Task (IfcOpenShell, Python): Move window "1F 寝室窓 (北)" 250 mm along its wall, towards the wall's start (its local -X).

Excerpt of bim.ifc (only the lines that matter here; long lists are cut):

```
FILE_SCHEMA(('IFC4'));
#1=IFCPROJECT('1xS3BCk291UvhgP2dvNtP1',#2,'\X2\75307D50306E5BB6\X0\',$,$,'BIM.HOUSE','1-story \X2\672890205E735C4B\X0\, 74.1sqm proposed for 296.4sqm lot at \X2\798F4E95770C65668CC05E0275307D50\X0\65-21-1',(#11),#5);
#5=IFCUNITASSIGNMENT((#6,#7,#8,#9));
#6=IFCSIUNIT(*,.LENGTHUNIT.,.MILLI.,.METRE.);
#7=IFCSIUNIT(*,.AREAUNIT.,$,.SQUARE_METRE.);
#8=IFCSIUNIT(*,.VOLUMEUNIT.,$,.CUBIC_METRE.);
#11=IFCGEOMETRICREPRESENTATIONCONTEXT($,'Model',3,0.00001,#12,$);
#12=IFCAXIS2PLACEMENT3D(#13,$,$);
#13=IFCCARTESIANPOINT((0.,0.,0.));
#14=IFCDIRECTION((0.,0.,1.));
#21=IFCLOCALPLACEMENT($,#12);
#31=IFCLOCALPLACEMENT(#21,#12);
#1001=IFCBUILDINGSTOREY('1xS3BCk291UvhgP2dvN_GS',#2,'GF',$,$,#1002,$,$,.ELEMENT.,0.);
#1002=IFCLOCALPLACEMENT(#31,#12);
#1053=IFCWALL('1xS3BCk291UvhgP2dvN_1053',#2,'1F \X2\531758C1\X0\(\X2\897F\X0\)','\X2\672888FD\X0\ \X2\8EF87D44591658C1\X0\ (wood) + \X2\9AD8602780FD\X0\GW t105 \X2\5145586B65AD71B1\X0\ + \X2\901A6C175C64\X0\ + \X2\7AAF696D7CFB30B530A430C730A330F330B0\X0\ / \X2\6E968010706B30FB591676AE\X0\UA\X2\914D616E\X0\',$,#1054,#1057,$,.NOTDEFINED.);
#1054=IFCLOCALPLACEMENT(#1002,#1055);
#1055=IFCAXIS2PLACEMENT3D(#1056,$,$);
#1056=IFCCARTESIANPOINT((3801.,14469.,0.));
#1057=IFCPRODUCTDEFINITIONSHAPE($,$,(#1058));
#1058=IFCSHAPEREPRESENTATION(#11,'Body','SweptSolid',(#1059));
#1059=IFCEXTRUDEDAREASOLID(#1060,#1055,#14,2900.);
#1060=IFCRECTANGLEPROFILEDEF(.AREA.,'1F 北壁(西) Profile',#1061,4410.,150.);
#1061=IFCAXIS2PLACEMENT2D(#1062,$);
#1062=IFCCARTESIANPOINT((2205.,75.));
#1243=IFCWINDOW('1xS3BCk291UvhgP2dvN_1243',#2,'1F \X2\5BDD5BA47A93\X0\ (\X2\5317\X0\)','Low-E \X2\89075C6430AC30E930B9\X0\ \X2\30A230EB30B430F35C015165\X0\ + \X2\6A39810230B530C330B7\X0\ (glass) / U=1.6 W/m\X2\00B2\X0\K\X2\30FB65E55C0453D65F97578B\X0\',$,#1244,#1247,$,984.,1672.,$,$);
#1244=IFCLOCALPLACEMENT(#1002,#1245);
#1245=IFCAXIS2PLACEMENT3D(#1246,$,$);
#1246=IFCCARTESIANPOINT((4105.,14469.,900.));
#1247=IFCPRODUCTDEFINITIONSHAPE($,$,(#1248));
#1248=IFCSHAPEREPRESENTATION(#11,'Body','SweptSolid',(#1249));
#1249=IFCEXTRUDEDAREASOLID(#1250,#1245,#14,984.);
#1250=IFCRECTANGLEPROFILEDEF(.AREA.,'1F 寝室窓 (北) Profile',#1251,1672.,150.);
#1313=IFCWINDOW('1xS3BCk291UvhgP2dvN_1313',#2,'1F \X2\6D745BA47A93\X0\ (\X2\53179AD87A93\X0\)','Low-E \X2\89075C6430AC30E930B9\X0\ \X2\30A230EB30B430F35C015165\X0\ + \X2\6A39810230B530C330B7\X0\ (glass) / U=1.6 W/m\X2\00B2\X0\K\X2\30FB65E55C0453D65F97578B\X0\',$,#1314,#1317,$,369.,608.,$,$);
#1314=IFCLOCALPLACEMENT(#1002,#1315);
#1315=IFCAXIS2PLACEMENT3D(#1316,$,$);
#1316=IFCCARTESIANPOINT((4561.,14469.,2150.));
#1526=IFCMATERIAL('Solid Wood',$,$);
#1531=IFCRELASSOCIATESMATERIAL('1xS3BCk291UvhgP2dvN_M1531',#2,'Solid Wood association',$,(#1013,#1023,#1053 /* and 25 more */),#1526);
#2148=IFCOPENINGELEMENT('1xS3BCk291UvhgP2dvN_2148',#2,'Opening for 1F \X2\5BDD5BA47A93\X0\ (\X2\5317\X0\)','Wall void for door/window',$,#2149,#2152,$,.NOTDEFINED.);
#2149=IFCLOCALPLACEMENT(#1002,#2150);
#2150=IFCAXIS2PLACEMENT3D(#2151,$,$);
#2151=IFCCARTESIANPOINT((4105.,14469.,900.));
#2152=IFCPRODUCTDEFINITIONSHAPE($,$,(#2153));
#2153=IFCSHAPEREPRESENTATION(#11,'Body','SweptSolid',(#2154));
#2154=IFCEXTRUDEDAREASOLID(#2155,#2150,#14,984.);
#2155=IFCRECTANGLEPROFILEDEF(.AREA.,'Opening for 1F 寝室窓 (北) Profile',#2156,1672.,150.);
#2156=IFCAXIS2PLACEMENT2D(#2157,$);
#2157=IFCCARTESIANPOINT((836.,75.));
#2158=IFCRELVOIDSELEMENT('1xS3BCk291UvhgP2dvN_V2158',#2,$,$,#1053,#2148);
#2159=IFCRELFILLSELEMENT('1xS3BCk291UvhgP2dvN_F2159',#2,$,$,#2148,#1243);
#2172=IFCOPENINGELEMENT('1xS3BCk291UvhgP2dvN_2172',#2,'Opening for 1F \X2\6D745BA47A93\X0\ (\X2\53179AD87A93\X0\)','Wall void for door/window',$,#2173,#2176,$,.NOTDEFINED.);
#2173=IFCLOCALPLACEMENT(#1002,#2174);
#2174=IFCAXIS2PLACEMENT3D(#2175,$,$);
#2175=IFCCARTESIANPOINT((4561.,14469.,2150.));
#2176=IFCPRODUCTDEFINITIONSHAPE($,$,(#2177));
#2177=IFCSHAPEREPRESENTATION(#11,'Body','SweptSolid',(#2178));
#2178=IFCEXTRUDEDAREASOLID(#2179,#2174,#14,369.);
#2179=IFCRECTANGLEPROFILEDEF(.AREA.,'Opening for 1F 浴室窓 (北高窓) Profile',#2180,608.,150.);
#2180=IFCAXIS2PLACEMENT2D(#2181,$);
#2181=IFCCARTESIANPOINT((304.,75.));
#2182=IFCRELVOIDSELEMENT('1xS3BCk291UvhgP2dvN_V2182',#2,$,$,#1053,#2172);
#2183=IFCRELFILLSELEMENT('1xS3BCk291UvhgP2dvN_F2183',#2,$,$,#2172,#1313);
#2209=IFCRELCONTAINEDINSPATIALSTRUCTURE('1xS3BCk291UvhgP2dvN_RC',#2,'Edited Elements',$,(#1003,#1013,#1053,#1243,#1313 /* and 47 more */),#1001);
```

```python
import ifcopenshell
import ifcopenshell.api.geometry
import ifcopenshell.util.placement
import ifcopenshell.util.unit

model = ifcopenshell.open("bim.ifc")
unit_scale = ifcopenshell.util.unit.calculate_unit_scale(model)

window = model.by_id(1243)
opening = window.FillsVoids[0].RelatingOpeningElement
wall = opening.VoidsElements[0].RelatingBuildingElement

wall_matrix = ifcopenshell.util.placement.get_local_placement(wall.ObjectPlacement)
shift = wall_matrix[:3, 0] * -0.25 / unit_scale
before = ifcopenshell.util.placement.get_local_placement(window.ObjectPlacement)[:3, 3].copy()

# The window is not placed relative to its opening, so move both.
for product in (opening, window):
    matrix = ifcopenshell.util.placement.get_local_placement(product.ObjectPlacement)
    matrix[:3, 3] += shift
    ifcopenshell.api.geometry.edit_object_placement(model, product=product, matrix=matrix, is_si=False)

after = ifcopenshell.util.placement.get_local_placement(window.ObjectPlacement)[:3, 3]
print("window moved by", (after - before).round(3) + 0.0)

model.write("bim-out.ifc")
```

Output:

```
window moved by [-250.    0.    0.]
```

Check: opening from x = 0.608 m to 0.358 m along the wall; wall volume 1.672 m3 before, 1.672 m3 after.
